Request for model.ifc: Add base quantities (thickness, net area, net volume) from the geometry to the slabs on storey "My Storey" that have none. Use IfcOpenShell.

First a look at what the model holds.

```python
import ifcopenshell
import ifcopenshell.util.element
import ifcopenshell.util.unit

model = ifcopenshell.open("model.ifc")
print(model.schema)
for unit_type in ("LENGTHUNIT", "AREAUNIT", "VOLUMEUNIT"):
    print(unit_type, ifcopenshell.util.unit.calculate_unit_scale(model, unit_type))
storey = next(s for s in model.by_type("IfcBuildingStorey") if s.Name == "My Storey")
slabs = [e for e in ifcopenshell.util.element.get_decomposition(storey) if e.is_a("IfcSlab")]
for e in sorted(slabs, key=lambda e: e.id()):
    print(e.id(), e.is_a(), e.Name, list(ifcopenshell.util.element.get_psets(e, qtos_only=True)), sep=" | ")
```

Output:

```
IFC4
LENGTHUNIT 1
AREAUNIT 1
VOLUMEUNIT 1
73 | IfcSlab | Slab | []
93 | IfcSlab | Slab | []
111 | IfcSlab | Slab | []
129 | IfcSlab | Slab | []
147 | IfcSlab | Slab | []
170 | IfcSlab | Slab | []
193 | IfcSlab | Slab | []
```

```python
import ifcopenshell
import ifcopenshell.api.pset
import ifcopenshell.geom
import ifcopenshell.util.element
import ifcopenshell.util.shape
import ifcopenshell.util.unit

model = ifcopenshell.open("model.ifc")
unit_scale = ifcopenshell.util.unit.calculate_unit_scale(model)
area_scale = ifcopenshell.util.unit.calculate_unit_scale(model, "AREAUNIT")
volume_scale = ifcopenshell.util.unit.calculate_unit_scale(model, "VOLUMEUNIT")
settings = ifcopenshell.geom.settings()

storey = next(s for s in model.by_type("IfcBuildingStorey") if s.Name == "My Storey")
slabs = [e for e in ifcopenshell.util.element.get_decomposition(storey) if e.is_a("IfcSlab")]

for e in sorted(slabs, key=lambda e: e.id()):
    if ifcopenshell.util.element.get_psets(e, qtos_only=True, should_inherit=False):
        continue
    # Geometry comes back in metres, in the element's own axes.
    shape = ifcopenshell.geom.create_shape(settings, e)
    values = {
        "Width": ifcopenshell.util.shape.get_z(shape.geometry) / unit_scale,
        "NetArea": ifcopenshell.util.shape.get_footprint_area(shape.geometry) / area_scale,
        "NetVolume": ifcopenshell.util.shape.get_volume(shape.geometry) / volume_scale,
    }
    qto = ifcopenshell.api.pset.add_qto(model, product=e, name="Qto_SlabBaseQuantities")
    ifcopenshell.api.pset.edit_qto(model, qto=qto, properties=values)
    print(e.id(), {k: round(v, 3) for k, v in values.items()})

model.write("model_rev.ifc")
```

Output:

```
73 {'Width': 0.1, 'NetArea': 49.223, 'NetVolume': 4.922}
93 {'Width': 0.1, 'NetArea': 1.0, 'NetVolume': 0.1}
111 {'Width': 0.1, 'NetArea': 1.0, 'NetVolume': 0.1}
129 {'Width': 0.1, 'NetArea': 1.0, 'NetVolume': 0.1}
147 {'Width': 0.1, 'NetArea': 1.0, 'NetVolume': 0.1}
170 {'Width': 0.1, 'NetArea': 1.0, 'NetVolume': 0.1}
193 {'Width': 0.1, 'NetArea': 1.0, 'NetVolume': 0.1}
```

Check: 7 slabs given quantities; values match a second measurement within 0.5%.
